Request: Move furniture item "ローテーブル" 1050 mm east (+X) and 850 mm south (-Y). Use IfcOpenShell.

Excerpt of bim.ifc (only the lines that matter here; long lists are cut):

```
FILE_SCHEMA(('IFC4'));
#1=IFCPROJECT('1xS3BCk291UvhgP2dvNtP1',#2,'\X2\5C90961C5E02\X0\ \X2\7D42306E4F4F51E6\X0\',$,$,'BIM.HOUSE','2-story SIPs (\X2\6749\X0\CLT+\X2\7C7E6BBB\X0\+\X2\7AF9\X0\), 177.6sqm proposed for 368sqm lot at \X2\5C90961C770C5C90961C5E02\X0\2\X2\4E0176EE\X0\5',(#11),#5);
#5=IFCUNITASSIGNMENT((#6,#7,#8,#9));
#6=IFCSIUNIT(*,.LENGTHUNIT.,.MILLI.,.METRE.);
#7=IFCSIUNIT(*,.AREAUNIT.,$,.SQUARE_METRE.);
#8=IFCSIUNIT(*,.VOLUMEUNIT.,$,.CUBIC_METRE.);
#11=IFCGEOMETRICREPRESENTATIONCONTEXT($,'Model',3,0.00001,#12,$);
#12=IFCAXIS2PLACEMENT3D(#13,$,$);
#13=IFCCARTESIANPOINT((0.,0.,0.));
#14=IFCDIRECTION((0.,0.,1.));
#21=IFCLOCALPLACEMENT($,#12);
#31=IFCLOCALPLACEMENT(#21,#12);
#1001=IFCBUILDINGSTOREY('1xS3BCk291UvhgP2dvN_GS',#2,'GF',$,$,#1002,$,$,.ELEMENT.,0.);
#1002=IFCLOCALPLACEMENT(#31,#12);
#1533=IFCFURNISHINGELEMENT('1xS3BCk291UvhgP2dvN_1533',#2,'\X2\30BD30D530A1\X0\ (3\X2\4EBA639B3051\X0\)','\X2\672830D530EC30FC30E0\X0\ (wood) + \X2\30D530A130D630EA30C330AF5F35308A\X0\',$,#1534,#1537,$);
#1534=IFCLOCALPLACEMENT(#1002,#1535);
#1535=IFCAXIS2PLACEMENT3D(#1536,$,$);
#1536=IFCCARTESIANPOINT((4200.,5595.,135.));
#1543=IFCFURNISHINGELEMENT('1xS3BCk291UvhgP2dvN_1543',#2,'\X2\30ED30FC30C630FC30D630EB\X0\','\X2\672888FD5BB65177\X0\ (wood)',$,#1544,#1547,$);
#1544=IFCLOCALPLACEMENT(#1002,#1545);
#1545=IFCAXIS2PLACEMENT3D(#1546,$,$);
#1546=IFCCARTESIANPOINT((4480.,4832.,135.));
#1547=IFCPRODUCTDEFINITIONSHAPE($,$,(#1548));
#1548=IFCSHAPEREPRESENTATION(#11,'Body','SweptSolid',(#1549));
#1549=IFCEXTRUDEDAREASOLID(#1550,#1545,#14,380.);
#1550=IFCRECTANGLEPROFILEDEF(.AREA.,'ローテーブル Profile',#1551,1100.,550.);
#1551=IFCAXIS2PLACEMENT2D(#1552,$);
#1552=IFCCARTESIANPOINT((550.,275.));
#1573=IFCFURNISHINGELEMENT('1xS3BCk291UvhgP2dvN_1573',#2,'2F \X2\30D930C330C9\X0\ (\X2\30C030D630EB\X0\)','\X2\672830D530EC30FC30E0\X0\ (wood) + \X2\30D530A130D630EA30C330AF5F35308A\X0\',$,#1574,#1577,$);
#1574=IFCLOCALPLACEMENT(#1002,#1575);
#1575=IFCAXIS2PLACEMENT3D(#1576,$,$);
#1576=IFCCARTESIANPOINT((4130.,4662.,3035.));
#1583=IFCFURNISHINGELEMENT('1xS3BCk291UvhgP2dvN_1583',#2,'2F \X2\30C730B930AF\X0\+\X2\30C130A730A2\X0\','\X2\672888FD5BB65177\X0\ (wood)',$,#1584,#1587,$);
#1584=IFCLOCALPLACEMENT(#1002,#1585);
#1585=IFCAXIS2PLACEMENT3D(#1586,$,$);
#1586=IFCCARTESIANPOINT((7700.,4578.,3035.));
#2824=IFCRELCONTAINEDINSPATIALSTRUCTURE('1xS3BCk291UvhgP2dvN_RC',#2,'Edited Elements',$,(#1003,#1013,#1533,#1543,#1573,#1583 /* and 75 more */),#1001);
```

```python
import ifcopenshell
import ifcopenshell.api.geometry
import ifcopenshell.util.placement

model = ifcopenshell.open("bim.ifc")

item = model.by_guid("1xS3BCk291UvhgP2dvN_1543")
matrix = ifcopenshell.util.placement.get_local_placement(item.ObjectPlacement)
matrix[0, 3] += 1050.0
matrix[1, 3] -= 850.0
ifcopenshell.api.geometry.edit_object_placement(model, product=item, matrix=matrix, is_si=False)

print(ifcopenshell.util.placement.get_local_placement(item.ObjectPlacement).round(3) + 0.0)

model.write("bim-out.ifc")
```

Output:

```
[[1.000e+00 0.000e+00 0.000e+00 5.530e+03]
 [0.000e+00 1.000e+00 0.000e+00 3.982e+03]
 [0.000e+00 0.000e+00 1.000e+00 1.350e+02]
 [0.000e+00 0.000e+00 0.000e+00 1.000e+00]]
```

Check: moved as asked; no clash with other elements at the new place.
